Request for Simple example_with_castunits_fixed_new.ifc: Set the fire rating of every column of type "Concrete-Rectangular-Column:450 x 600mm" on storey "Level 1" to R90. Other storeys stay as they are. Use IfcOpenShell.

First a look at what the model holds.

```python
import ifcopenshell
import ifcopenshell.util.element

model = ifcopenshell.open("Simple example_with_castunits_fixed_new.ifc")
print(model.schema)
storey = next(s for s in model.by_type("IfcBuildingStorey") if s.Name == "Level 1")
columns = [e for e in ifcopenshell.util.element.get_decomposition(storey) if e.is_a("IfcColumn")]
seen = {}
for e in columns:
    element_type = ifcopenshell.util.element.get_type(e)
    key = (element_type.Name if element_type != e and element_type else None, ifcopenshell.util.element.get_pset(e, "Pset_ColumnCommon", "FireRating"))
    seen[key] = seen.get(key, 0) + 1
for (name, value), count in sorted(seen.items(), key=str):
    print(count, "x", name, "|", value)
```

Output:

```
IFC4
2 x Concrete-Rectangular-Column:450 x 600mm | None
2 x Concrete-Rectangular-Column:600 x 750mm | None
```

```python
import ifcopenshell
import ifcopenshell.api.pset
import ifcopenshell.util.element

model = ifcopenshell.open("Simple example_with_castunits_fixed_new.ifc")

storey = next(s for s in model.by_type("IfcBuildingStorey") if s.Name == "Level 1")
columns = [e for e in ifcopenshell.util.element.get_decomposition(storey) if e.is_a("IfcColumn")]

count = 0
for e in columns:
    element_type = ifcopenshell.util.element.get_type(e)
    if element_type in (None, e) or element_type.Name != "Concrete-Rectangular-Column:450 x 600mm":
        continue
    # add_pset returns the element's existing set when there is one.
    pset = ifcopenshell.api.pset.add_pset(model, product=e, name="Pset_ColumnCommon")
    ifcopenshell.api.pset.edit_pset(model, pset=pset, properties={"FireRating": "R90"})
    count += 1

print(count, "columns updated")

model.write("Simple example_with_castunits_fixed_new-out.ifc")
```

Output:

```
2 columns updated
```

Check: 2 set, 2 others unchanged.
